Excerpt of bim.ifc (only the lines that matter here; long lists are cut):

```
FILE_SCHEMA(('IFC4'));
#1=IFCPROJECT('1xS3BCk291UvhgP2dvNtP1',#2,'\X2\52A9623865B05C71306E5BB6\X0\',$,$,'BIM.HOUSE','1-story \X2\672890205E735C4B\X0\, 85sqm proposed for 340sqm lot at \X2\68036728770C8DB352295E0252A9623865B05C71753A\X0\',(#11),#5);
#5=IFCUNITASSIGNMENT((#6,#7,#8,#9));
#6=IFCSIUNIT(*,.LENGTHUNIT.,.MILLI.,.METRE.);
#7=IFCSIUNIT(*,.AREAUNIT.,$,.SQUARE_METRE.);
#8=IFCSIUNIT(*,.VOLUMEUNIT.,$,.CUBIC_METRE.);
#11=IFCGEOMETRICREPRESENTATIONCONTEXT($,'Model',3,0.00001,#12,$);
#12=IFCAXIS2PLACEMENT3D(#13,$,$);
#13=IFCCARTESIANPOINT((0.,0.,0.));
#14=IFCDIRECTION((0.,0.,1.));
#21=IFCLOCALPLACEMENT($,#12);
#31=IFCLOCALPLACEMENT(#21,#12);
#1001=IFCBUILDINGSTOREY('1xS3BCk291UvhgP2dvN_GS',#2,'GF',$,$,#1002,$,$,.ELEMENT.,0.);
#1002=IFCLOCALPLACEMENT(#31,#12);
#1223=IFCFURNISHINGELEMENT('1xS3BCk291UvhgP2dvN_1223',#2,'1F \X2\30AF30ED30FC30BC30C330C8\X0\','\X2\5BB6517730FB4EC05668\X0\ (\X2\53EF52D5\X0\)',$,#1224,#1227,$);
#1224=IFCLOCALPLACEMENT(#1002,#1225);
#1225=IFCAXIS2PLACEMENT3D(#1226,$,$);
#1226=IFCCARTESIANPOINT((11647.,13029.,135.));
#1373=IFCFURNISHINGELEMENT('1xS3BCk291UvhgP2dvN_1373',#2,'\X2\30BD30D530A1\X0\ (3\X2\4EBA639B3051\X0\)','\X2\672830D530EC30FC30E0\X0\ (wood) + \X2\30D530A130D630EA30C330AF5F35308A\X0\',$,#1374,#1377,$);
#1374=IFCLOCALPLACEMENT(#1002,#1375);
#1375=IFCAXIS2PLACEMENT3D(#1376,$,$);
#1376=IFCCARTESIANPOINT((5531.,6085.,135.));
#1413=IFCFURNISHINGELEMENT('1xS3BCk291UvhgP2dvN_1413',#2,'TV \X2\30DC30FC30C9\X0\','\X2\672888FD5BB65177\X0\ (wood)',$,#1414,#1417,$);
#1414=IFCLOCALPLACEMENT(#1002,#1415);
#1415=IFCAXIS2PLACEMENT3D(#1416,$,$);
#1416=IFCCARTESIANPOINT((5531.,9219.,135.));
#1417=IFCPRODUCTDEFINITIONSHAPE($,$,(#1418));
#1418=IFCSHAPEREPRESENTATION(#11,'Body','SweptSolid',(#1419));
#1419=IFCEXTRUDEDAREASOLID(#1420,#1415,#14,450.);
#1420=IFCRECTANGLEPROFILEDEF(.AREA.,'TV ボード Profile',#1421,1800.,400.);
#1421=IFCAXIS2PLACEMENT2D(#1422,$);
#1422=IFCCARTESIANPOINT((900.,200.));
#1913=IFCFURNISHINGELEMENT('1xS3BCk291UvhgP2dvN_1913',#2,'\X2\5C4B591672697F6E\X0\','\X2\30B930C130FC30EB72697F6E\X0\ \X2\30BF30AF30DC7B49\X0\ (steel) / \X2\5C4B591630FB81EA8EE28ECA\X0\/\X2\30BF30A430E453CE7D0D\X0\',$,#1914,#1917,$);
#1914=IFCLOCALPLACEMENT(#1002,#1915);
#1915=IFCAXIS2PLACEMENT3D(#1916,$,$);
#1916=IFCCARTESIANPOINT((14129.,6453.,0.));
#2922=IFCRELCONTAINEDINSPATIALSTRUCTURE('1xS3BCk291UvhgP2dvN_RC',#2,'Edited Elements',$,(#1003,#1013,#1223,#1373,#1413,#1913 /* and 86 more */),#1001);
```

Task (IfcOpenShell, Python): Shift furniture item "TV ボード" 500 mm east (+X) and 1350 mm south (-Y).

```python
import ifcopenshell
import ifcopenshell.api.geometry
import ifcopenshell.util.placement
import ifcopenshell.util.unit

model = ifcopenshell.open("bim.ifc")
unit_scale = ifcopenshell.util.unit.calculate_unit_scale(model)

item = model.by_guid("1xS3BCk291UvhgP2dvN_1413")
matrix = ifcopenshell.util.placement.get_local_placement(item.ObjectPlacement)
matrix[0, 3] += 0.5 / unit_scale
matrix[1, 3] -= 1.35 / unit_scale
ifcopenshell.api.geometry.edit_object_placement(model, product=item, matrix=matrix, is_si=False)

print(ifcopenshell.util.placement.get_local_placement(item.ObjectPlacement).round(3) + 0.0)

model.write("bim-out.ifc")
```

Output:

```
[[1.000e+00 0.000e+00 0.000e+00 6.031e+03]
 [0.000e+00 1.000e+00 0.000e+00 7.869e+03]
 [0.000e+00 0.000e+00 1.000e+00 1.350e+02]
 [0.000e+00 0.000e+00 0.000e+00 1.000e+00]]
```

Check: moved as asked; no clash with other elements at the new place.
